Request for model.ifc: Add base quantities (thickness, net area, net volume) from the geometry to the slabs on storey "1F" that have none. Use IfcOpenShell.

First a look at what the model holds.

```python
import ifcopenshell
import ifcopenshell.util.element
import ifcopenshell.util.unit

model = ifcopenshell.open("model.ifc")
print(model.schema)
for unit_type in ("LENGTHUNIT", "AREAUNIT", "VOLUMEUNIT"):
    print(unit_type, ifcopenshell.util.unit.calculate_unit_scale(model, unit_type))
storey = next(s for s in model.by_type("IfcBuildingStorey") if s.Name == "1F")
slabs = [e for e in ifcopenshell.util.element.get_decomposition(storey) if e.is_a("IfcSlab")]
for e in sorted(slabs, key=lambda e: e.id()):
    print(e.id(), e.is_a(), e.Name, list(ifcopenshell.util.element.get_psets(e, qtos_only=True)), sep=" | ")
```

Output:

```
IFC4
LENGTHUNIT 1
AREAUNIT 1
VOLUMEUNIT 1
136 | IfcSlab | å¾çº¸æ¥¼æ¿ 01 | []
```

```python
import ifcopenshell
import ifcopenshell.api.pset
import ifcopenshell.geom
import ifcopenshell.util.element
import ifcopenshell.util.shape
import ifcopenshell.util.unit

model = ifcopenshell.open("model.ifc")
unit_scale = ifcopenshell.util.unit.calculate_unit_scale(model)
area_scale = ifcopenshell.util.unit.calculate_unit_scale(model, "AREAUNIT")
volume_scale = ifcopenshell.util.unit.calculate_unit_scale(model, "VOLUMEUNIT")
settings = ifcopenshell.geom.settings()

storey = next(s for s in model.by_type("IfcBuildingStorey") if s.Name == "1F")
slabs = [e for e in ifcopenshell.util.element.get_decomposition(storey) if e.is_a("IfcSlab")]

for e in sorted(slabs, key=lambda e: e.id()):
    if ifcopenshell.util.element.get_psets(e, qtos_only=True, should_inherit=False):
        continue
    # Geometry comes back in metres, in the element's own axes.
    shape = ifcopenshell.geom.create_shape(settings, e)
    values = {
        "Width": ifcopenshell.util.shape.get_z(shape.geometry) / unit_scale,
        "NetArea": ifcopenshell.util.shape.get_footprint_area(shape.geometry) / area_scale,
        "NetVolume": ifcopenshell.util.shape.get_volume(shape.geometry) / volume_scale,
    }
    qto = ifcopenshell.api.pset.add_qto(model, product=e, name="Qto_SlabBaseQuantities")
    ifcopenshell.api.pset.edit_qto(model, qto=qto, properties=values)
    print(e.id(), {k: round(v, 3) for k, v in values.items()})

model.write("model-out.ifc")
```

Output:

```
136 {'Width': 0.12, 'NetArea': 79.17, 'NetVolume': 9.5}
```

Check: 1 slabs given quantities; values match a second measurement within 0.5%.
